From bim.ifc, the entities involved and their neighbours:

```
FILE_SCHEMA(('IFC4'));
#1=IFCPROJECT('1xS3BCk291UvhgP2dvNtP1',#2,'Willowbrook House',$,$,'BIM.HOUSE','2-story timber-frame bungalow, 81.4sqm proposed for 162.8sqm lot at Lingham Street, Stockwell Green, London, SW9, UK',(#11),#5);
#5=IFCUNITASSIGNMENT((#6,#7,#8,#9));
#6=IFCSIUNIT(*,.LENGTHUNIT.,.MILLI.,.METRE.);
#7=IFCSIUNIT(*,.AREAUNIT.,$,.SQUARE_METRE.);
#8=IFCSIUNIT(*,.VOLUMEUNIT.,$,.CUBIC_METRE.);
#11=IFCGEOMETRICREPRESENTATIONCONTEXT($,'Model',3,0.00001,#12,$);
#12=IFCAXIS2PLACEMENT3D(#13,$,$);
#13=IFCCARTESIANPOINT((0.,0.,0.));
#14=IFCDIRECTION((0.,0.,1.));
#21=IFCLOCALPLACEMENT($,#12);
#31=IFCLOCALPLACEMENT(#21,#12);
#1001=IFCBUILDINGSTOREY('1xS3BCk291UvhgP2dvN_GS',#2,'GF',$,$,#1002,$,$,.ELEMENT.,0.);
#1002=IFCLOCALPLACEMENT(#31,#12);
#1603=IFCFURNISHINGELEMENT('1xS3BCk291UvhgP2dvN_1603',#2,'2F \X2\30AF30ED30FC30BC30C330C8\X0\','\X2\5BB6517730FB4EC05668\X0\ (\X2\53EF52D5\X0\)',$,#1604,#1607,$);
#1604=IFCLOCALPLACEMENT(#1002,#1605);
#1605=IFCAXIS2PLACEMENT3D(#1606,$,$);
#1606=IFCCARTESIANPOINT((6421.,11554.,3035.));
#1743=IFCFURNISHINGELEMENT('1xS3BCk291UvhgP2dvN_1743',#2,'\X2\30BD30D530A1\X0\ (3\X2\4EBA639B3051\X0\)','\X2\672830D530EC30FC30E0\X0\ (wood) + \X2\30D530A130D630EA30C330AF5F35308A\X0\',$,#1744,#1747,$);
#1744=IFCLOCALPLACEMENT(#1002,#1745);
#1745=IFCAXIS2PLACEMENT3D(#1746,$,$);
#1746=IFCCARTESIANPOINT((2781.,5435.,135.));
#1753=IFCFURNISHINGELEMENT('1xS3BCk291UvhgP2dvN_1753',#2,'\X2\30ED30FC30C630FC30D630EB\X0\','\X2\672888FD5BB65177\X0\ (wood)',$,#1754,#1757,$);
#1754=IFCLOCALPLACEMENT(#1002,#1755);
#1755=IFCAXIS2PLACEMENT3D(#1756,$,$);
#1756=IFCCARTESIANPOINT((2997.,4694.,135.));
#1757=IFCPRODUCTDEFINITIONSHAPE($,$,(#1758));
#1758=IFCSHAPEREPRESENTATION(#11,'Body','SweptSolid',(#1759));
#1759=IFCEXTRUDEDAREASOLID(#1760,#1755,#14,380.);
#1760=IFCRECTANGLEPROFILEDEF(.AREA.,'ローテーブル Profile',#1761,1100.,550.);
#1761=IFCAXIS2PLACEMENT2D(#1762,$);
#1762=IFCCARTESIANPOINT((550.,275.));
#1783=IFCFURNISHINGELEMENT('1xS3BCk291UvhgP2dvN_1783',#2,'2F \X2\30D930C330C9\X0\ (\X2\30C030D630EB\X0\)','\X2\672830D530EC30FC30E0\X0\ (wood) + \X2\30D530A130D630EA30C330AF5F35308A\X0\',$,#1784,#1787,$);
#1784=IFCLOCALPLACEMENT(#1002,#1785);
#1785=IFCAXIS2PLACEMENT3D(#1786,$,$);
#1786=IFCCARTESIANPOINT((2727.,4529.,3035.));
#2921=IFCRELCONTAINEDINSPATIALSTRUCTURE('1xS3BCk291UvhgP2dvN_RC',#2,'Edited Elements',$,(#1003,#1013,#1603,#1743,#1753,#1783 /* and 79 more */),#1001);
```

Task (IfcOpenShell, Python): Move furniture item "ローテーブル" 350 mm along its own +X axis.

```python
import ifcopenshell
import ifcopenshell.api.geometry
import ifcopenshell.util.placement

model = ifcopenshell.open("bim.ifc")

item = model.by_guid("1xS3BCk291UvhgP2dvN_1753")
matrix = ifcopenshell.util.placement.get_local_placement(item.ObjectPlacement)
matrix[:3, 3] += matrix[:3, 0] * 350.0
ifcopenshell.api.geometry.edit_object_placement(model, product=item, matrix=matrix, is_si=False)

print(ifcopenshell.util.placement.get_local_placement(item.ObjectPlacement).round(3) + 0.0)

model.write("bim_rev.ifc")
```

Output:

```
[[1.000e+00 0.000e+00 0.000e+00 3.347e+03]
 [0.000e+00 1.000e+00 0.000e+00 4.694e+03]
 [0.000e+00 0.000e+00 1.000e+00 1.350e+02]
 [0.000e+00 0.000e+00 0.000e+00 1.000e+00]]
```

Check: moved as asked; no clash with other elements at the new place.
